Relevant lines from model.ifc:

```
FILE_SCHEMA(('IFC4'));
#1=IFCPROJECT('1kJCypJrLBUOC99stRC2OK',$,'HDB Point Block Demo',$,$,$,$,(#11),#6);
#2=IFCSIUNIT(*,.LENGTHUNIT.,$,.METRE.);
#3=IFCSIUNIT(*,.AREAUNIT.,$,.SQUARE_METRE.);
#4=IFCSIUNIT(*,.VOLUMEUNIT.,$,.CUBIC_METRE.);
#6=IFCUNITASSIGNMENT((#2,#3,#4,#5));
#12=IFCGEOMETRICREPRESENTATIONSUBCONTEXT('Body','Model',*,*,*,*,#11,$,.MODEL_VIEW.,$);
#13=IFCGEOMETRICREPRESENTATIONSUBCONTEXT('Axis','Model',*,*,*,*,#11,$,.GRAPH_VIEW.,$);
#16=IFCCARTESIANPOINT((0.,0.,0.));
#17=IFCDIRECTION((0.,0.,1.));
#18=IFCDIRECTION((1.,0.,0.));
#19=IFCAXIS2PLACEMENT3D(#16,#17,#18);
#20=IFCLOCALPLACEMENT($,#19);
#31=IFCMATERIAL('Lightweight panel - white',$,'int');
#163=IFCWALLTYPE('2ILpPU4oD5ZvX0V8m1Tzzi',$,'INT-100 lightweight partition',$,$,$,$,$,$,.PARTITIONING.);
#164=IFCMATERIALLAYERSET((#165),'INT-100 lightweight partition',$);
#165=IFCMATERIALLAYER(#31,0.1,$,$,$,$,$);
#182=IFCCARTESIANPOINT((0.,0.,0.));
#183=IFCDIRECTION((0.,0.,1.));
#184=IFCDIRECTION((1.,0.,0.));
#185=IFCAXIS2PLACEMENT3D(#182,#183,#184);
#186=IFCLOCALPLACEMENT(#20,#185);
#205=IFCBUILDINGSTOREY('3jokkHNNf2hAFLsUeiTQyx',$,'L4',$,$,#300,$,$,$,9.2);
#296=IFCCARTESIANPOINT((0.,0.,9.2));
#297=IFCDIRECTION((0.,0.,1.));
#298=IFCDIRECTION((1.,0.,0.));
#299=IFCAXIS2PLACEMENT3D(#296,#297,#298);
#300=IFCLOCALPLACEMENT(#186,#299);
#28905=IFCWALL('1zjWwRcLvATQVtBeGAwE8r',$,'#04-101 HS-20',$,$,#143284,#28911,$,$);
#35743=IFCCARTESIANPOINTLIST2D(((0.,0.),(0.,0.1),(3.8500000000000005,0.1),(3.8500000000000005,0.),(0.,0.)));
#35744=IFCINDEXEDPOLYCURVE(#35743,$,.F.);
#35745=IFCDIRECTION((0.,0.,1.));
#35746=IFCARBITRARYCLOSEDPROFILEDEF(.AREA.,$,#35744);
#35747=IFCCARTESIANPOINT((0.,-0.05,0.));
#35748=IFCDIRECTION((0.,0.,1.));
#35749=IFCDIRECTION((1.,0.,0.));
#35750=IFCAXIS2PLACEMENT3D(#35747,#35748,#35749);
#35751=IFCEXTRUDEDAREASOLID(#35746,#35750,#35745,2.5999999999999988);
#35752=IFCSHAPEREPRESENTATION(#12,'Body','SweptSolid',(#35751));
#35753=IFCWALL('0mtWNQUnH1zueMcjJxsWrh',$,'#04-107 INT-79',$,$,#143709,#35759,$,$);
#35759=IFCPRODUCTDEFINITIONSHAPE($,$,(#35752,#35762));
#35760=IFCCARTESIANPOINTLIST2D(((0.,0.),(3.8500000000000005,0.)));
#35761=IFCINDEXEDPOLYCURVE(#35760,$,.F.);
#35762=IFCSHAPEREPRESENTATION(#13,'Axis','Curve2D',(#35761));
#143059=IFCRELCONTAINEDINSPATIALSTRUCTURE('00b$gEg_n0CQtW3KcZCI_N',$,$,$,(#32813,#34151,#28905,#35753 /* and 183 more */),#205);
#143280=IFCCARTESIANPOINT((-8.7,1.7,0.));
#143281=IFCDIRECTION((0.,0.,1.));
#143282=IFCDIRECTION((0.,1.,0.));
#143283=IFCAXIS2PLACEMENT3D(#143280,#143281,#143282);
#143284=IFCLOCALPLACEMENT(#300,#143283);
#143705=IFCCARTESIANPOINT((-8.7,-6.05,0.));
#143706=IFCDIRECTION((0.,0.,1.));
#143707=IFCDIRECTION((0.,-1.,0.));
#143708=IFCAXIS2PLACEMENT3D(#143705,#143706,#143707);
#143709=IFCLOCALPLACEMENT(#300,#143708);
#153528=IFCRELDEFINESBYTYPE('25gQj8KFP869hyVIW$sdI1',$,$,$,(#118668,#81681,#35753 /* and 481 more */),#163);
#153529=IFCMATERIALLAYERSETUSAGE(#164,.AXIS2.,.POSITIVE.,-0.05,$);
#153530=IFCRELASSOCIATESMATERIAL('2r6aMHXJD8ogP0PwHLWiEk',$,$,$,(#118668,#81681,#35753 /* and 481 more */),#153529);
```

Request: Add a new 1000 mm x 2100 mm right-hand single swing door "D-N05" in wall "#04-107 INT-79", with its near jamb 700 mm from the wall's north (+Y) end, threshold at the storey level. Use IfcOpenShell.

```python
import numpy as np
import ifcopenshell
import ifcopenshell.api.feature
import ifcopenshell.api.geometry
import ifcopenshell.api.root
import ifcopenshell.api.spatial
import ifcopenshell.geom
import ifcopenshell.util.element
import ifcopenshell.util.placement
import ifcopenshell.util.representation
import ifcopenshell.util.shape
import ifcopenshell.util.unit

model = ifcopenshell.open("model.ifc")
unit_scale = ifcopenshell.util.unit.calculate_unit_scale(model)
settings = ifcopenshell.geom.settings()


def volume(element):
    """Net volume in cubic metres, openings subtracted."""
    shape = ifcopenshell.geom.create_shape(settings, element)
    return ifcopenshell.util.shape.get_volume(shape.geometry)


wall = model.by_id(35753)
storey = ifcopenshell.util.element.get_container(wall, ifc_class="IfcBuildingStorey")
context = ifcopenshell.util.representation.get_context(model, "Model", "Body", "MODEL_VIEW")
before = volume(wall)

width, height, from_end, sill = 1, 2.1, 0.7, 0.0  # metres

# The wall runs along its own X axis, and the end named is its -X end.
wall_shape = ifcopenshell.geom.create_shape(settings, wall)
x, y, z = ifcopenshell.util.shape.get_vertices(wall_shape.geometry).T
start = x.min() + from_end
face, thickness = float(y.min()), float(y.max() - y.min())
wall_matrix = ifcopenshell.util.placement.get_local_placement(wall.ObjectPlacement)
level = ifcopenshell.util.placement.get_local_placement(storey.ObjectPlacement)[2, 3]


def in_wall(x, y):
    """Placement at x, y metres in the wall's axes, at sill height."""
    matrix = wall_matrix.copy()
    matrix[:, 3] = wall_matrix @ np.array([x / unit_scale, y / unit_scale, 0.0, 1.0])
    matrix[2, 3] = level + sill / unit_scale
    return matrix


# Opening: a box that overshoots both wall faces by 50 mm.
opening = ifcopenshell.api.root.create_entity(model, ifc_class="IfcOpeningElement", predefined_type="OPENING")
box = ifcopenshell.api.geometry.add_wall_representation(
    model, context=context, length=width, height=height, thickness=thickness + 0.1
)
ifcopenshell.api.geometry.assign_representation(model, product=opening, representation=box)
ifcopenshell.api.geometry.edit_object_placement(model, product=opening, matrix=in_wall(start, face - 0.05), is_si=False)
ifcopenshell.api.feature.add_feature(model, feature=opening, element=wall)

door = ifcopenshell.api.root.create_entity(model, ifc_class="IfcDoor", name="D-N05", predefined_type="DOOR")
door.OverallWidth, door.OverallHeight = width / unit_scale, height / unit_scale
door.OperationType = "SINGLE_SWING_RIGHT"
body = ifcopenshell.api.geometry.add_door_representation(
    model,
    context=context,
    overall_width=door.OverallWidth,
    overall_height=door.OverallHeight,
    operation_type="SINGLE_SWING_RIGHT",
    lining_properties={"LiningDepth": thickness / unit_scale, "ThresholdDepth": thickness / unit_scale},
)
ifcopenshell.api.geometry.assign_representation(model, product=door, representation=body)
ifcopenshell.api.spatial.assign_container(model, products=[door], relating_structure=storey)
ifcopenshell.api.feature.add_filling(model, opening=opening, element=door)

# The lining spans the wall, so the door starts at the wall face.
ifcopenshell.api.geometry.edit_object_placement(model, product=door, matrix=in_wall(start, face), is_si=False)

after = volume(wall)

print(f"wall volume {before:.3f} -> {after:.3f} m3")

model.write("model_v2.ifc")
```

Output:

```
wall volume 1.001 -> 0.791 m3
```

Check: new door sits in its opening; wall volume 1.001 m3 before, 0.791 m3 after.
